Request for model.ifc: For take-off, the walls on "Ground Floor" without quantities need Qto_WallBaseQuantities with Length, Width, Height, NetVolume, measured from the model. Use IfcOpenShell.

First a look at what the model holds.

```python
import ifcopenshell
import ifcopenshell.util.element
import ifcopenshell.util.unit

model = ifcopenshell.open("model.ifc")
print(model.schema)
for unit_type in ("LENGTHUNIT", "AREAUNIT", "VOLUMEUNIT"):
    print(unit_type, ifcopenshell.util.unit.calculate_unit_scale(model, unit_type))
storey = next(s for s in model.by_type("IfcBuildingStorey") if s.Name == "Ground Floor")
walls = [e for e in ifcopenshell.util.element.get_decomposition(storey) if e.is_a("IfcWall")]
for e in sorted(walls, key=lambda e: e.id()):
    print(e.id(), e.is_a(), e.Name, list(ifcopenshell.util.element.get_psets(e, qtos_only=True)), sep=" | ")
```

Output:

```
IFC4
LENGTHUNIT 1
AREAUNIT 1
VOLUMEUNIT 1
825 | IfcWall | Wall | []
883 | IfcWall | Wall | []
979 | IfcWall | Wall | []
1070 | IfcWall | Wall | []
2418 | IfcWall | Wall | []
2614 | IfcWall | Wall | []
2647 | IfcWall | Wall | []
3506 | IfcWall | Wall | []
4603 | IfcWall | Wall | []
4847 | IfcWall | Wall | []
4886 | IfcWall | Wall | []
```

```python
import ifcopenshell
import ifcopenshell.api.pset
import ifcopenshell.geom
import ifcopenshell.util.element
import ifcopenshell.util.shape
import ifcopenshell.util.unit

model = ifcopenshell.open("model.ifc")
unit_scale = ifcopenshell.util.unit.calculate_unit_scale(model)
volume_scale = ifcopenshell.util.unit.calculate_unit_scale(model, "VOLUMEUNIT")
settings = ifcopenshell.geom.settings()

storey = next(s for s in model.by_type("IfcBuildingStorey") if s.Name == "Ground Floor")
walls = [e for e in ifcopenshell.util.element.get_decomposition(storey) if e.is_a("IfcWall")]

for e in sorted(walls, key=lambda e: e.id()):
    if ifcopenshell.util.element.get_psets(e, qtos_only=True, should_inherit=False):
        continue
    # Geometry comes back in metres, in the element's own axes.
    shape = ifcopenshell.geom.create_shape(settings, e)
    values = {
        "Length": ifcopenshell.util.shape.get_x(shape.geometry) / unit_scale,
        "Width": ifcopenshell.util.shape.get_y(shape.geometry) / unit_scale,
        "Height": ifcopenshell.util.shape.get_z(shape.geometry) / unit_scale,
        "NetVolume": ifcopenshell.util.shape.get_volume(shape.geometry) / volume_scale,
    }
    qto = ifcopenshell.api.pset.add_qto(model, product=e, name="Qto_WallBaseQuantities")
    ifcopenshell.api.pset.edit_qto(model, qto=qto, properties=values)
    print(e.id(), {k: round(v, 3) for k, v in values.items()})

model.write("model-out.ifc")
```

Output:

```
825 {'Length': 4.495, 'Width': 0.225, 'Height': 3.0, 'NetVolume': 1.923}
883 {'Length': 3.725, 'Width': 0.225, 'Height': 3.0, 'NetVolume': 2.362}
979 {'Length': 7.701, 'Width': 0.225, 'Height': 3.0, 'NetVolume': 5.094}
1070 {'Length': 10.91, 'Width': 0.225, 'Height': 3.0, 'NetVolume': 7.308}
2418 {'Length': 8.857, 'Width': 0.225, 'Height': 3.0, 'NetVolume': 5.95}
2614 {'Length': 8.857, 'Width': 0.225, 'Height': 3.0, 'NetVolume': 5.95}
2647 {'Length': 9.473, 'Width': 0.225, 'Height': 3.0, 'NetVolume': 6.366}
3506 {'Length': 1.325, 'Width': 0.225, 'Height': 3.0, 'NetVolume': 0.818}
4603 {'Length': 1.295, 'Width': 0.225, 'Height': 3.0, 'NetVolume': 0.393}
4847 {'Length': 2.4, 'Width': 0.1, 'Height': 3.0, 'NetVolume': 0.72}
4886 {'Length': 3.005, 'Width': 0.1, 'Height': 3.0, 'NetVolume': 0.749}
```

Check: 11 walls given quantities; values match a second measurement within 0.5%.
